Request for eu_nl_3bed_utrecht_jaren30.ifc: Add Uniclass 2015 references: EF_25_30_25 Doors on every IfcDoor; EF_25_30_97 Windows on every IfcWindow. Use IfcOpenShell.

First a look at what the model holds.

```python
import ifcopenshell

model = ifcopenshell.open("eu_nl_3bed_utrecht_jaren30.ifc")
print(model.schema)
print("classifications:", [c.Name for c in model.by_type("IfcClassification")])
for ifc_class in ("IfcDoor", "IfcRoof", "IfcStair", "IfcWall", "IfcWindow"):
    print(ifc_class, len(model.by_type(ifc_class)))
```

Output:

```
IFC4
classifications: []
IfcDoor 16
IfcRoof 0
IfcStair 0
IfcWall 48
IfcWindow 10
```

```python
import ifcopenshell
import ifcopenshell.api.classification

model = ifcopenshell.open("eu_nl_3bed_utrecht_jaren30.ifc")

system = ifcopenshell.api.classification.add_classification(model, classification="Uniclass 2015")

codes = {
    "IfcDoor": ("EF_25_30_25", "Doors"),
    "IfcWindow": ("EF_25_30_97", "Windows"),
}
for ifc_class, (code, name) in codes.items():
    products = model.by_type(ifc_class)
    ifcopenshell.api.classification.add_reference(
        model, products=products, classification=system, identification=code, name=name
    )
    print(code, len(products))

model.write("eu_nl_3bed_utrecht_jaren30_v2.ifc")
```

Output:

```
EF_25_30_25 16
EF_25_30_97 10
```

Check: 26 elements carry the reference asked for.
